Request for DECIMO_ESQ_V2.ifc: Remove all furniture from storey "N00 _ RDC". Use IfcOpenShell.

First a look at what the model holds.

```python
import ifcopenshell
import ifcopenshell.util.element

model = ifcopenshell.open("DECIMO_ESQ_V2.ifc")
print(model.schema)
storey = next(s for s in model.by_type("IfcBuildingStorey") if s.Name == "N00 _ RDC")
furniture = [e for e in ifcopenshell.util.element.get_decomposition(storey) if e.is_a("IfcFurnishingElement")]
seen = {}
for e in furniture:
    element_type = ifcopenshell.util.element.get_type(e)
    name = element_type.Name if element_type not in (None, e) else None
    seen[name] = seen.get(name, 0) + 1
for name, count in sorted(seen.items(), key=str):
    print(count, "x", name)
```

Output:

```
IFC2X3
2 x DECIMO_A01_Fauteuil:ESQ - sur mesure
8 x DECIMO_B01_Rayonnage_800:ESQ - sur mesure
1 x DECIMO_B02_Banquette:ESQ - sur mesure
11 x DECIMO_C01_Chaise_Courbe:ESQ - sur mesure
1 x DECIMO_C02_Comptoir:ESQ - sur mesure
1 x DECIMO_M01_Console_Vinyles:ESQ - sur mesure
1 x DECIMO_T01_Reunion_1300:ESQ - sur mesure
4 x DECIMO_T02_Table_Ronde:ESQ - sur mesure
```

```python
import ifcopenshell
import ifcopenshell.api.root
import ifcopenshell.util.element

model = ifcopenshell.open("DECIMO_ESQ_V2.ifc")

storey = next(s for s in model.by_type("IfcBuildingStorey") if s.Name == "N00 _ RDC")
furniture = [e for e in ifcopenshell.util.element.get_decomposition(storey) if e.is_a("IfcFurnishingElement")]

for e in furniture:
    ifcopenshell.api.root.remove_product(model, product=e)
print(len(furniture), "removed")

model.write("DECIMO_ESQ_V2_rev.ifc")
```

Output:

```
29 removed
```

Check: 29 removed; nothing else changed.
